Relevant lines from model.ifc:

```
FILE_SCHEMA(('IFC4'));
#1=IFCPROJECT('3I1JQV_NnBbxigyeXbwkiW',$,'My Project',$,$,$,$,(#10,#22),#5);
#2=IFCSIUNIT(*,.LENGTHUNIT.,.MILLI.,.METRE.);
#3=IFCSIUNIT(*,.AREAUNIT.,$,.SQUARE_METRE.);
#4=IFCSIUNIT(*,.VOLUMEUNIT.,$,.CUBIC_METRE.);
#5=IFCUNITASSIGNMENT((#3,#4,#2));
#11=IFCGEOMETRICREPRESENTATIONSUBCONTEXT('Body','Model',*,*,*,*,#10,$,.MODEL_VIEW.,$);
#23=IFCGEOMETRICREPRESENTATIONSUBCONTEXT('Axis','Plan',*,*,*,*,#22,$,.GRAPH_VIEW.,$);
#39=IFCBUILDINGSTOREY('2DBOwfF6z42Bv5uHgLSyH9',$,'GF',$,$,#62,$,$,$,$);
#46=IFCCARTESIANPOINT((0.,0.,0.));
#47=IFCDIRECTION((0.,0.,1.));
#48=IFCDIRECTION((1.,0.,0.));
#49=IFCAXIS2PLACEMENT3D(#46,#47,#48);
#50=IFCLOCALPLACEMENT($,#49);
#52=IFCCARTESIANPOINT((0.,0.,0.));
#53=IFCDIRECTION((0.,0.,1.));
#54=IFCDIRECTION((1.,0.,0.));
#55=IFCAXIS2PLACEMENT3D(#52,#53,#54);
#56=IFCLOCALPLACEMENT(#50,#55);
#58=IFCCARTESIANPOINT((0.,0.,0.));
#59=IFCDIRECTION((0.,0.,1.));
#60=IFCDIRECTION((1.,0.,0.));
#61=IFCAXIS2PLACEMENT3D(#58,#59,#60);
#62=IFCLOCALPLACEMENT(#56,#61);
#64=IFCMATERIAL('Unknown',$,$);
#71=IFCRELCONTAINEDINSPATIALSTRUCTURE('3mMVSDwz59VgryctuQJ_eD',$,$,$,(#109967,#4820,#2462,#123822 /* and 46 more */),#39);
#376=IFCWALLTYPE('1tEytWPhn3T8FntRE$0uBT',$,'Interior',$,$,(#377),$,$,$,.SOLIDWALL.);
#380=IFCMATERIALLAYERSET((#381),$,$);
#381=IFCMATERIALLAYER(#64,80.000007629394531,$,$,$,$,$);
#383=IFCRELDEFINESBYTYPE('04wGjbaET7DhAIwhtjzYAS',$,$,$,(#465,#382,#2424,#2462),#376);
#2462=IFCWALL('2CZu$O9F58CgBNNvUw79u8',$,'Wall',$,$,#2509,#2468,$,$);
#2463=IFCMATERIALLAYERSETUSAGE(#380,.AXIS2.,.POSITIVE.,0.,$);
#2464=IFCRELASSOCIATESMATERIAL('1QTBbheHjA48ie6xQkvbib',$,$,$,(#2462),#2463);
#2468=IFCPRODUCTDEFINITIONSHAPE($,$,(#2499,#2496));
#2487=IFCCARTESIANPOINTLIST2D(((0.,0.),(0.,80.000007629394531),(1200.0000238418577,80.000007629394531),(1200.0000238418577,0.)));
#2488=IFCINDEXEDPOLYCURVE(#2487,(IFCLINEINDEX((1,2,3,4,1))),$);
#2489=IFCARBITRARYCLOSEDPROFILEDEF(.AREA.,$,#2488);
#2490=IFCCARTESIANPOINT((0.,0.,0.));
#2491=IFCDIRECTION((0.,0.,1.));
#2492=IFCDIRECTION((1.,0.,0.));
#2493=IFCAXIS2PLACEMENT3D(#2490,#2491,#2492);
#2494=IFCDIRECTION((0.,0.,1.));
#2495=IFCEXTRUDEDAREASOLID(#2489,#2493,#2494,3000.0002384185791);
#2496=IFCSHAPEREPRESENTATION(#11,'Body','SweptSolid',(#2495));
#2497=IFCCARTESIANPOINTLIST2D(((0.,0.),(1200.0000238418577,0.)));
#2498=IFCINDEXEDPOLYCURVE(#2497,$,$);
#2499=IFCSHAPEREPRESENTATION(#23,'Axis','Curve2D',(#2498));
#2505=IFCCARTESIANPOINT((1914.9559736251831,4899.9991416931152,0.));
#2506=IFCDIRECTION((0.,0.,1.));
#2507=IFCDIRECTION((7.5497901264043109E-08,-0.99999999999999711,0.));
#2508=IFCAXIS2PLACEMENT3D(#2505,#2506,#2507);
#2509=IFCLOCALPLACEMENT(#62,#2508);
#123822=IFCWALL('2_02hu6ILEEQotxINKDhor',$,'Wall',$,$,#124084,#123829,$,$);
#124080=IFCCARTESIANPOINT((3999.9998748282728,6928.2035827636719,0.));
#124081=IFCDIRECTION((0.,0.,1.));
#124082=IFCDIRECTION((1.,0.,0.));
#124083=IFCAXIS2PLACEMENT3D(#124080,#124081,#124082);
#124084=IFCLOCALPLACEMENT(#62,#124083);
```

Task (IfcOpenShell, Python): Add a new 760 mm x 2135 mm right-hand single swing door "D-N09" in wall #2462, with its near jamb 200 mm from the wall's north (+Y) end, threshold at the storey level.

```python
import numpy as np
import ifcopenshell
import ifcopenshell.api.feature
import ifcopenshell.api.geometry
import ifcopenshell.api.root
import ifcopenshell.api.spatial
import ifcopenshell.geom
import ifcopenshell.util.element
import ifcopenshell.util.placement
import ifcopenshell.util.representation
import ifcopenshell.util.shape
import ifcopenshell.util.unit

model = ifcopenshell.open("model.ifc")
unit_scale = ifcopenshell.util.unit.calculate_unit_scale(model)
settings = ifcopenshell.geom.settings()


def volume(element):
    """Net volume in cubic metres, openings subtracted."""
    shape = ifcopenshell.geom.create_shape(settings, element)
    return ifcopenshell.util.shape.get_volume(shape.geometry)


wall = model.by_guid("2CZu$O9F58CgBNNvUw79u8")
storey = ifcopenshell.util.element.get_container(wall, ifc_class="IfcBuildingStorey")
context = ifcopenshell.util.representation.get_context(model, "Model", "Body", "MODEL_VIEW")
before = volume(wall)

width, height, from_end, sill = 0.76, 2.135, 0.2, 0.0  # metres

# The wall runs along its own X axis, and the end named is its -X end.
wall_shape = ifcopenshell.geom.create_shape(settings, wall)
x, y, z = ifcopenshell.util.shape.get_vertices(wall_shape.geometry).T
start = x.min() + from_end
face, thickness = float(y.min()), float(y.max() - y.min())
wall_matrix = ifcopenshell.util.placement.get_local_placement(wall.ObjectPlacement)
level = ifcopenshell.util.placement.get_local_placement(storey.ObjectPlacement)[2, 3]


def in_wall(x, y):
    """Placement at x, y metres in the wall's axes, at sill height."""
    matrix = wall_matrix.copy()
    matrix[:, 3] = wall_matrix @ np.array([x / unit_scale, y / unit_scale, 0.0, 1.0])
    matrix[2, 3] = level + sill / unit_scale
    return matrix


# Opening: a box that overshoots both wall faces by 50 mm.
opening = ifcopenshell.api.root.create_entity(model, ifc_class="IfcOpeningElement", predefined_type="OPENING")
box = ifcopenshell.api.geometry.add_wall_representation(
    model, context=context, length=width, height=height, thickness=thickness + 0.1
)
ifcopenshell.api.geometry.assign_representation(model, product=opening, representation=box)
ifcopenshell.api.geometry.edit_object_placement(model, product=opening, matrix=in_wall(start, face - 0.05), is_si=False)
ifcopenshell.api.feature.add_feature(model, feature=opening, element=wall)

door = ifcopenshell.api.root.create_entity(model, ifc_class="IfcDoor", name="D-N09", predefined_type="DOOR")
door.OverallWidth, door.OverallHeight = width / unit_scale, height / unit_scale
door.OperationType = "SINGLE_SWING_RIGHT"
body = ifcopenshell.api.geometry.add_door_representation(
    model,
    context=context,
    overall_width=door.OverallWidth,
    overall_height=door.OverallHeight,
    operation_type="SINGLE_SWING_RIGHT",
    lining_properties={"LiningDepth": thickness / unit_scale, "ThresholdDepth": thickness / unit_scale},
)
ifcopenshell.api.geometry.assign_representation(model, product=door, representation=body)
ifcopenshell.api.spatial.assign_container(model, products=[door], relating_structure=storey)
ifcopenshell.api.feature.add_filling(model, opening=opening, element=door)

# The lining spans the wall, so the door starts at the wall face.
ifcopenshell.api.geometry.edit_object_placement(model, product=door, matrix=in_wall(start, face), is_si=False)

after = volume(wall)

print(f"wall volume {before:.3f} -> {after:.3f} m3")

model.write("model-out.ifc")
```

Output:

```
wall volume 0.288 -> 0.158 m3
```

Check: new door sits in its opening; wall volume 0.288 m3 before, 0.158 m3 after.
